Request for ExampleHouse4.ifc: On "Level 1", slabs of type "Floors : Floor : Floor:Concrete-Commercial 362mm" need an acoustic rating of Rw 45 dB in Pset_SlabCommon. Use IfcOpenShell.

First a look at what the model holds.

```python
import ifcopenshell
import ifcopenshell.util.element

model = ifcopenshell.open("ExampleHouse4.ifc")
print(model.schema)
storey = next(s for s in model.by_type("IfcBuildingStorey") if s.Name == "Level 1")
slabs = [e for e in ifcopenshell.util.element.get_decomposition(storey) if e.is_a("IfcSlab")]
seen = {}
for e in slabs:
    element_type = ifcopenshell.util.element.get_type(e)
    key = (element_type.Name if element_type != e and element_type else None, ifcopenshell.util.element.get_pset(e, "Pset_SlabCommon", "AcousticRating"))
    seen[key] = seen.get(key, 0) + 1
for (name, value), count in sorted(seen.items(), key=str):
    print(count, "x", name, "|", value)
```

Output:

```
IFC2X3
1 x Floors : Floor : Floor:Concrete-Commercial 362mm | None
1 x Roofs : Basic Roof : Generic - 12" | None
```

```python
import ifcopenshell
import ifcopenshell.api.pset
import ifcopenshell.util.element

model = ifcopenshell.open("ExampleHouse4.ifc")

storey = next(s for s in model.by_type("IfcBuildingStorey") if s.Name == "Level 1")
slabs = [e for e in ifcopenshell.util.element.get_decomposition(storey) if e.is_a("IfcSlab")]

count = 0
for e in slabs:
    element_type = ifcopenshell.util.element.get_type(e)
    if element_type in (None, e) or element_type.Name != "Floors : Floor : Floor:Concrete-Commercial 362mm":
        continue
    # add_pset returns the element's existing set when there is one.
    pset = ifcopenshell.api.pset.add_pset(model, product=e, name="Pset_SlabCommon")
    ifcopenshell.api.pset.edit_pset(model, pset=pset, properties={"AcousticRating": "Rw 45 dB"})
    count += 1

print(count, "slabs updated")

model.write("ExampleHouse4_updated.ifc")
```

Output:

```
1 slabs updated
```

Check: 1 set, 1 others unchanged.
